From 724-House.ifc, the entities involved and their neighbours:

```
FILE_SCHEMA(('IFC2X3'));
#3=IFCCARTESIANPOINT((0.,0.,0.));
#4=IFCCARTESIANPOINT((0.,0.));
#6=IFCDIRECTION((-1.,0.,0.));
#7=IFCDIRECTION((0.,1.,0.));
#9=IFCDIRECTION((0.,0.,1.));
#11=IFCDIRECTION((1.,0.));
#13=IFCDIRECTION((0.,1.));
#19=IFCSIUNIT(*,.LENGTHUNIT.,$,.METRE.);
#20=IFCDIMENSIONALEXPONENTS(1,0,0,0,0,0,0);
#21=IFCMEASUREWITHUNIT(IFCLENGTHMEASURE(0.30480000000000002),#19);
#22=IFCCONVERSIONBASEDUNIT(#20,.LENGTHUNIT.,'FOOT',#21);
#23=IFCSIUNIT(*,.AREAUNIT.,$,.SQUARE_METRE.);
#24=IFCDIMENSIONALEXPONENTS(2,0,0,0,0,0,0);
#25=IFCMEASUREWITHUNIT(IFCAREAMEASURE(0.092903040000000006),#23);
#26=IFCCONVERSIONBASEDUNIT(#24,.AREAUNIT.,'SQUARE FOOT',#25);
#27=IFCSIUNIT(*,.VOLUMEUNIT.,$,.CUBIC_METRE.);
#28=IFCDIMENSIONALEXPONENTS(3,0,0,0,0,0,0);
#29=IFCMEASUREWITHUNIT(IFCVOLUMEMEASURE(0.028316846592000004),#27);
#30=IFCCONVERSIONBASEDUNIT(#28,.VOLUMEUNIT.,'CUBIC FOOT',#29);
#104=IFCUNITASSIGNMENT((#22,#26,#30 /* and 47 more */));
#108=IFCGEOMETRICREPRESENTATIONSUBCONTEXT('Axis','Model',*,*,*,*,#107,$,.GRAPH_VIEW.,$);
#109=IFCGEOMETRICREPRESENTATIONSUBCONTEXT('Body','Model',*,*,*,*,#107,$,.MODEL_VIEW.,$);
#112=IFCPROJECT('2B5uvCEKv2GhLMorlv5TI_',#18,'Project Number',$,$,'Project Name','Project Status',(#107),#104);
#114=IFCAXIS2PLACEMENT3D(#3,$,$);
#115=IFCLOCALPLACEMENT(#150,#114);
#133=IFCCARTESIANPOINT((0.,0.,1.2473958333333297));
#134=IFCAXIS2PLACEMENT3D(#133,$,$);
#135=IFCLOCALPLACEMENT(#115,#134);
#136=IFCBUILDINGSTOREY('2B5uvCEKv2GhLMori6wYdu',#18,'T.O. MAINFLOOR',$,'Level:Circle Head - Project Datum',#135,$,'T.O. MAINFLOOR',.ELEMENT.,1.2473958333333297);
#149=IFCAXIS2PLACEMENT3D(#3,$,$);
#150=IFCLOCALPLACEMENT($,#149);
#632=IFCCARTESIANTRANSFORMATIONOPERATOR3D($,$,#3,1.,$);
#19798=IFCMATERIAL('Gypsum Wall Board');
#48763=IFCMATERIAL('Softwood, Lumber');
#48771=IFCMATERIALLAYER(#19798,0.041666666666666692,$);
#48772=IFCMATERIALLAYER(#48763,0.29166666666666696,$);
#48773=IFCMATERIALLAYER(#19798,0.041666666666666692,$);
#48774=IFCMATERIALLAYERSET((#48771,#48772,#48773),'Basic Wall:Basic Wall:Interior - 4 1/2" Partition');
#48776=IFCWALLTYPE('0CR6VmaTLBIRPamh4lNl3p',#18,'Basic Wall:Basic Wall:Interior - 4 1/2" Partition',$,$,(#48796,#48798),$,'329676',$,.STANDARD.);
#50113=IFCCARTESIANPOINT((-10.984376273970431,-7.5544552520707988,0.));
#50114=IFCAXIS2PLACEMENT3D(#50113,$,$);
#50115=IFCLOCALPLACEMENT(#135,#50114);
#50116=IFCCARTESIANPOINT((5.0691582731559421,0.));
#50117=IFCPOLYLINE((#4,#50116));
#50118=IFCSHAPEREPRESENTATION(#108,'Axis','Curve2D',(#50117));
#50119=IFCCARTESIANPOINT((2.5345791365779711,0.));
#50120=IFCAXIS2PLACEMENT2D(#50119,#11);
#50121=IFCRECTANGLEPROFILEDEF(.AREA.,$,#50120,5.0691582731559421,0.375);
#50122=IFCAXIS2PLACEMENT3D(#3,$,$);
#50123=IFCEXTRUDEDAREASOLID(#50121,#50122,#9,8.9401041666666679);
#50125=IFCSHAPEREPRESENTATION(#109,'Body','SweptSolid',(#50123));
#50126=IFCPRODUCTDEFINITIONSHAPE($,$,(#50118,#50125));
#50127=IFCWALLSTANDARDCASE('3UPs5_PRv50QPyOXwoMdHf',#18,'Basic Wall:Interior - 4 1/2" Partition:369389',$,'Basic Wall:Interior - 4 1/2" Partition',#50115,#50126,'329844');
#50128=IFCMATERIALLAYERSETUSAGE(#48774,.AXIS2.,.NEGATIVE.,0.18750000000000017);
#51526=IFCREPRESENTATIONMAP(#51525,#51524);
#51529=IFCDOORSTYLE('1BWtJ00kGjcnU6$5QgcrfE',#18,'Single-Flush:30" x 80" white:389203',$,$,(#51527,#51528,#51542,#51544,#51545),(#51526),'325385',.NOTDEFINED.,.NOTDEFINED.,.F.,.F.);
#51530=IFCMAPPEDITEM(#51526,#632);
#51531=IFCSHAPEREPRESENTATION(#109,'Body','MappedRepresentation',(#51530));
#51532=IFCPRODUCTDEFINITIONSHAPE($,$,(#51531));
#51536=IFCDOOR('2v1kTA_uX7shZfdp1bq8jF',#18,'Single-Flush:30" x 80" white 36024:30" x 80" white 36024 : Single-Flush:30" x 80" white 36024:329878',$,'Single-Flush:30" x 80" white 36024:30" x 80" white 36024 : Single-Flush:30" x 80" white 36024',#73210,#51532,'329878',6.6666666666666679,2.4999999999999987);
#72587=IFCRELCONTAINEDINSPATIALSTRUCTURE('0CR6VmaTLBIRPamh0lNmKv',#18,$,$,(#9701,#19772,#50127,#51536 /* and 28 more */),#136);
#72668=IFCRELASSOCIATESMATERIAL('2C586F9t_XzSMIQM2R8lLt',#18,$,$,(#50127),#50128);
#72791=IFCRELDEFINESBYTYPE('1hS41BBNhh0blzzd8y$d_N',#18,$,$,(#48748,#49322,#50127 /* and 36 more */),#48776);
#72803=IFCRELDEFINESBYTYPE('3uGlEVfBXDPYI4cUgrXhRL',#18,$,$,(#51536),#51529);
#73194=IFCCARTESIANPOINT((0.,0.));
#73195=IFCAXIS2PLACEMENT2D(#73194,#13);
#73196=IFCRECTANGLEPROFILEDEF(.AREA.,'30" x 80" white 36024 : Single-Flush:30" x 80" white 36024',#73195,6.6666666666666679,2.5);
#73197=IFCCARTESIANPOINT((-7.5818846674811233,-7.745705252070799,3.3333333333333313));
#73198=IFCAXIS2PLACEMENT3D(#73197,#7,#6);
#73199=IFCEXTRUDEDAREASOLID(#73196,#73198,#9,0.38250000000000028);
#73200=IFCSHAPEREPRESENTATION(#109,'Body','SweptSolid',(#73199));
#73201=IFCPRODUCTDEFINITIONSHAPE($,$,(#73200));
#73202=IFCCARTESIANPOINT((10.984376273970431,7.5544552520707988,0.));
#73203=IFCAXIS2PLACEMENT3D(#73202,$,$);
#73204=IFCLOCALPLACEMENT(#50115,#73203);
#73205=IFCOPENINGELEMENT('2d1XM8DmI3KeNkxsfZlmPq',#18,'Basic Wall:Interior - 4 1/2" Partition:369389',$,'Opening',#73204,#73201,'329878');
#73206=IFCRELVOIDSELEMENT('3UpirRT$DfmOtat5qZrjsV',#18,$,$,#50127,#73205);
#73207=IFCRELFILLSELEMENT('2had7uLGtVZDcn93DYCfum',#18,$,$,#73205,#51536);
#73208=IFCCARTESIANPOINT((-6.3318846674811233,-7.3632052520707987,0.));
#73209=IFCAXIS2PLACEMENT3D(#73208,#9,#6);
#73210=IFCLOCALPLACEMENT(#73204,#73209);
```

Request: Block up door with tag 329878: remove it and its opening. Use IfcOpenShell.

```python
import ifcopenshell
import ifcopenshell.api.feature
import ifcopenshell.api.root
import ifcopenshell.geom
import ifcopenshell.util.shape

model = ifcopenshell.open("724-House.ifc")
settings = ifcopenshell.geom.settings()


def volume(element):
    """Net volume in cubic metres, openings subtracted."""
    shape = ifcopenshell.geom.create_shape(settings, element)
    return ifcopenshell.util.shape.get_volume(shape.geometry)


door = model.by_guid("2v1kTA_uX7shZfdp1bq8jF")
opening = door.FillsVoids[0].RelatingOpeningElement
wall = opening.VoidsElements[0].RelatingBuildingElement
before = volume(wall)

ifcopenshell.api.root.remove_product(model, product=door)
ifcopenshell.api.feature.remove_feature(model, feature=opening)

after = volume(wall)

print(f"wall volume {before:.3f} -> {after:.3f} m3")

model.write("724-House_edited.ifc")
```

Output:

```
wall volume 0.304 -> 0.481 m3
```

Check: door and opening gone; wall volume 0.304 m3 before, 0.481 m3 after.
